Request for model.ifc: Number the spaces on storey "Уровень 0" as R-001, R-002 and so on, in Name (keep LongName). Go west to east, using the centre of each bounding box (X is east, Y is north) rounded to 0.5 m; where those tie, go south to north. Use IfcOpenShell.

First a look at what the model holds.

```python
import ifcopenshell
import ifcopenshell.util.element
import ifcopenshell.util.placement

model = ifcopenshell.open("model.ifc")
print(model.schema)
storey = next(s for s in model.by_type("IfcBuildingStorey") if s.Name == "Уровень 0")
spaces = [e for e in ifcopenshell.util.element.get_decomposition(storey) if e.is_a("IfcSpace")]
for e in sorted(spaces, key=lambda e: e.id()):
    origin = ifcopenshell.util.placement.get_local_placement(e.ObjectPlacement)[:3, 3]
    print(e.id(), e.Name, e.LongName, origin.round(2) + 0.0, sep=" | ")
```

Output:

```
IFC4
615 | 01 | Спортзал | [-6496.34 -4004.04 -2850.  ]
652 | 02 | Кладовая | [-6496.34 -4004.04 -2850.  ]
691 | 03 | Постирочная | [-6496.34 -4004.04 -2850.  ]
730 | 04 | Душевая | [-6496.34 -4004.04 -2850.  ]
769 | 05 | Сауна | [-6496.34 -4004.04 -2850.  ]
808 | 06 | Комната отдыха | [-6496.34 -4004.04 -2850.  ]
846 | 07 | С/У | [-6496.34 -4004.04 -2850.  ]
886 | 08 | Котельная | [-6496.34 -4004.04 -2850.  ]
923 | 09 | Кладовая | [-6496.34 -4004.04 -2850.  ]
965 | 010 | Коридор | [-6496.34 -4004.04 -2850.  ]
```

```python
import ifcopenshell
import ifcopenshell.geom
import ifcopenshell.util.element
import ifcopenshell.util.shape

model = ifcopenshell.open("model.ifc")
settings = ifcopenshell.geom.settings()
settings.set("use-world-coords", True)


def centre(element):
    shape = ifcopenshell.geom.create_shape(settings, element)
    return ifcopenshell.util.shape.get_bbox_centroid(shape.geometry)


storey = next(s for s in model.by_type("IfcBuildingStorey") if s.Name == "Уровень 0")
spaces = [e for e in ifcopenshell.util.element.get_decomposition(storey) if e.is_a("IfcSpace")]

# Insertion points can sit at a corner or the storey origin, so sort by the geometry (in metres).
centres = {e: centre(e) for e in spaces}
spaces.sort(key=lambda e: (round(centres[e][0] / 0.5), centres[e][1]))

for i, e in enumerate(spaces, start=1):
    number = f"R-0{i:02d}"
    e.Name = number
    print(e.id(), number)

model.write("model-out.ifc")
```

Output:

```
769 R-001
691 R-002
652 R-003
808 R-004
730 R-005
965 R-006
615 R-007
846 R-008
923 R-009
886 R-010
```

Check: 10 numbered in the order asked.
